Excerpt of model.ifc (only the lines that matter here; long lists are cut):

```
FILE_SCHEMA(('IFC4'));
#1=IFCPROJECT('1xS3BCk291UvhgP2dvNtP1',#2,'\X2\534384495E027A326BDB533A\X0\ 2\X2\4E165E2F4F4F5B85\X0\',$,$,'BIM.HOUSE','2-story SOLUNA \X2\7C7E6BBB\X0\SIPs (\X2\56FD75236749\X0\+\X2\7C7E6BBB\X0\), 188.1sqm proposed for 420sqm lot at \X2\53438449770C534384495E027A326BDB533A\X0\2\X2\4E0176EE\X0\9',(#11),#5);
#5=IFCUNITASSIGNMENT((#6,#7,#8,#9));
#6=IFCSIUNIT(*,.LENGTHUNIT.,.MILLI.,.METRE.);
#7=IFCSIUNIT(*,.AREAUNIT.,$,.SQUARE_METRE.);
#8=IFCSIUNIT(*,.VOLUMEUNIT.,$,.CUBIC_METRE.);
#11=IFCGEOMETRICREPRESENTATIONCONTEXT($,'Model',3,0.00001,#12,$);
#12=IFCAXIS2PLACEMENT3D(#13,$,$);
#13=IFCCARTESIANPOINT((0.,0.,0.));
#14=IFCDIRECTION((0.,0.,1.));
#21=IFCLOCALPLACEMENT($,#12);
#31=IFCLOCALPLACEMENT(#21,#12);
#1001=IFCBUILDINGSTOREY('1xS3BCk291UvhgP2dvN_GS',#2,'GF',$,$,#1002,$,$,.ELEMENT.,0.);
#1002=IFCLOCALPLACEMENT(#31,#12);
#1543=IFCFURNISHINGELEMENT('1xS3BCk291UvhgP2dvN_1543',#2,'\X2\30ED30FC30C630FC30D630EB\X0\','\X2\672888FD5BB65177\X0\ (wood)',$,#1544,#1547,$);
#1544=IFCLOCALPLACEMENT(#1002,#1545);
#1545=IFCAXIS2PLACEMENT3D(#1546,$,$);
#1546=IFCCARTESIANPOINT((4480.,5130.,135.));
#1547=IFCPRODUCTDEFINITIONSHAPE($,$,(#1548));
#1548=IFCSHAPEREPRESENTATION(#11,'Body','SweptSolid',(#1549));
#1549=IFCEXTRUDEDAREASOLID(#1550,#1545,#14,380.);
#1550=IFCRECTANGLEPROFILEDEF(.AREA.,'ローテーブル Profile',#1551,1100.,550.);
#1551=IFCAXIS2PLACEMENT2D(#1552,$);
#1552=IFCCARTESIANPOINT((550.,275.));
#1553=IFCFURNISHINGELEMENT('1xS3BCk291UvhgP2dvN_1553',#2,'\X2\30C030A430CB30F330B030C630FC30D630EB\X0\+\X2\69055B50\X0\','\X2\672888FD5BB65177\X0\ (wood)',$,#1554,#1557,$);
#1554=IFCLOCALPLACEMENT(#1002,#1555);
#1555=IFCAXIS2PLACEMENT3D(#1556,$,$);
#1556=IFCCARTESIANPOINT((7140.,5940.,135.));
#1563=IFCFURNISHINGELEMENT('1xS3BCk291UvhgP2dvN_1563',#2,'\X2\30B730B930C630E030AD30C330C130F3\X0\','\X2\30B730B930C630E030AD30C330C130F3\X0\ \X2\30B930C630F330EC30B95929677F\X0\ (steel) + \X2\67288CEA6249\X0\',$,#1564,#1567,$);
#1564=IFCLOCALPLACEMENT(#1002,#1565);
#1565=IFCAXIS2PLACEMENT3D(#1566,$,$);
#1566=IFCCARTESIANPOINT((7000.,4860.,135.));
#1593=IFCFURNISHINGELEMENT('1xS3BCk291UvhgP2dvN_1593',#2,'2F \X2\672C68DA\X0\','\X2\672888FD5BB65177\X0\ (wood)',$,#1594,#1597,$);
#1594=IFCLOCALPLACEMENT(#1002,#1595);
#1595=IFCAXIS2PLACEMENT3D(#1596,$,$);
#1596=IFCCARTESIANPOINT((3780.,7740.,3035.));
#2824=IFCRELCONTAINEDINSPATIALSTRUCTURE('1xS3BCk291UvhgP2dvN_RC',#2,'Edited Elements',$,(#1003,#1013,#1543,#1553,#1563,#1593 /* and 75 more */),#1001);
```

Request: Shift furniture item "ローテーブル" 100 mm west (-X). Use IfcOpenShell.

```python
import ifcopenshell
import ifcopenshell.api.geometry
import ifcopenshell.util.placement

model = ifcopenshell.open("model.ifc")

item = model.by_id(1543)
matrix = ifcopenshell.util.placement.get_local_placement(item.ObjectPlacement)
matrix[0, 3] -= 100.0
ifcopenshell.api.geometry.edit_object_placement(model, product=item, matrix=matrix, is_si=False)

print(ifcopenshell.util.placement.get_local_placement(item.ObjectPlacement).round(3) + 0.0)

model.write("model_rev.ifc")
```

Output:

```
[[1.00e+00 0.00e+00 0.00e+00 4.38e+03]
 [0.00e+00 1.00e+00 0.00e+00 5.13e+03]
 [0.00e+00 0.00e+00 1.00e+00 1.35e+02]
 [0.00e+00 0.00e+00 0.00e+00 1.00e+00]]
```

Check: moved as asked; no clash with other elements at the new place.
